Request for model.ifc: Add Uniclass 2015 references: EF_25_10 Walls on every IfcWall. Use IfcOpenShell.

First a look at what the model holds.

```python
import ifcopenshell

model = ifcopenshell.open("model.ifc")
print(model.schema)
print("classifications:", [c.Name for c in model.by_type("IfcClassification")])
for ifc_class in ("IfcDoor", "IfcRoof", "IfcStair", "IfcWall", "IfcWindow"):
    print(ifc_class, len(model.by_type(ifc_class)))
```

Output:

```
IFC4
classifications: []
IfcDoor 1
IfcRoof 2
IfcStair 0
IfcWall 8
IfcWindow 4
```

```python
import ifcopenshell
import ifcopenshell.api.classification

model = ifcopenshell.open("model.ifc")

system = ifcopenshell.api.classification.add_classification(model, classification="Uniclass 2015")

codes = {
    "IfcWall": ("EF_25_10", "Walls"),
}
for ifc_class, (code, name) in codes.items():
    products = model.by_type(ifc_class)
    ifcopenshell.api.classification.add_reference(
        model, products=products, classification=system, identification=code, name=name
    )
    print(code, len(products))

model.write("model_rev.ifc")
```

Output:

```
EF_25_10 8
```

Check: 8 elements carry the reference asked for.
